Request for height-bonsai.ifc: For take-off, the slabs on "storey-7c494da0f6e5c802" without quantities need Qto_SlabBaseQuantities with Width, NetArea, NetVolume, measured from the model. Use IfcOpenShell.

First a look at what the model holds.

```python
import ifcopenshell
import ifcopenshell.util.element
import ifcopenshell.util.unit

model = ifcopenshell.open("height-bonsai.ifc")
print(model.schema)
for unit_type in ("LENGTHUNIT", "AREAUNIT", "VOLUMEUNIT"):
    print(unit_type, ifcopenshell.util.unit.calculate_unit_scale(model, unit_type))
storey = next(s for s in model.by_type("IfcBuildingStorey") if s.Name == "storey-7c494da0f6e5c802")
slabs = [e for e in ifcopenshell.util.element.get_decomposition(storey) if e.is_a("IfcSlab")]
for e in sorted(slabs, key=lambda e: e.id()):
    print(e.id(), e.is_a(), e.Name, list(ifcopenshell.util.element.get_psets(e, qtos_only=True)), sep=" | ")
```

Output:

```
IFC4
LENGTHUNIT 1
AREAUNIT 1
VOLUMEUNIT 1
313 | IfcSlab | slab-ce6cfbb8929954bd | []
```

```python
import ifcopenshell
import ifcopenshell.api.pset
import ifcopenshell.geom
import ifcopenshell.util.element
import ifcopenshell.util.shape
import ifcopenshell.util.unit

model = ifcopenshell.open("height-bonsai.ifc")
unit_scale = ifcopenshell.util.unit.calculate_unit_scale(model)
area_scale = ifcopenshell.util.unit.calculate_unit_scale(model, "AREAUNIT")
volume_scale = ifcopenshell.util.unit.calculate_unit_scale(model, "VOLUMEUNIT")
settings = ifcopenshell.geom.settings()

storey = next(s for s in model.by_type("IfcBuildingStorey") if s.Name == "storey-7c494da0f6e5c802")
slabs = [e for e in ifcopenshell.util.element.get_decomposition(storey) if e.is_a("IfcSlab")]

for e in sorted(slabs, key=lambda e: e.id()):
    if ifcopenshell.util.element.get_psets(e, qtos_only=True, should_inherit=False):
        continue
    # Geometry comes back in metres, in the element's own axes.
    shape = ifcopenshell.geom.create_shape(settings, e)
    values = {
        "Width": ifcopenshell.util.shape.get_z(shape.geometry) / unit_scale,
        "NetArea": ifcopenshell.util.shape.get_footprint_area(shape.geometry) / area_scale,
        "NetVolume": ifcopenshell.util.shape.get_volume(shape.geometry) / volume_scale,
    }
    qto = ifcopenshell.api.pset.add_qto(model, product=e, name="Qto_SlabBaseQuantities")
    ifcopenshell.api.pset.edit_qto(model, qto=qto, properties=values)
    print(e.id(), {k: round(v, 3) for k, v in values.items()})

model.write("height-bonsai-out.ifc")
```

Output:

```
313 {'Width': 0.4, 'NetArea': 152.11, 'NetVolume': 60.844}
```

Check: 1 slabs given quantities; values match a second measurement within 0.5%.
